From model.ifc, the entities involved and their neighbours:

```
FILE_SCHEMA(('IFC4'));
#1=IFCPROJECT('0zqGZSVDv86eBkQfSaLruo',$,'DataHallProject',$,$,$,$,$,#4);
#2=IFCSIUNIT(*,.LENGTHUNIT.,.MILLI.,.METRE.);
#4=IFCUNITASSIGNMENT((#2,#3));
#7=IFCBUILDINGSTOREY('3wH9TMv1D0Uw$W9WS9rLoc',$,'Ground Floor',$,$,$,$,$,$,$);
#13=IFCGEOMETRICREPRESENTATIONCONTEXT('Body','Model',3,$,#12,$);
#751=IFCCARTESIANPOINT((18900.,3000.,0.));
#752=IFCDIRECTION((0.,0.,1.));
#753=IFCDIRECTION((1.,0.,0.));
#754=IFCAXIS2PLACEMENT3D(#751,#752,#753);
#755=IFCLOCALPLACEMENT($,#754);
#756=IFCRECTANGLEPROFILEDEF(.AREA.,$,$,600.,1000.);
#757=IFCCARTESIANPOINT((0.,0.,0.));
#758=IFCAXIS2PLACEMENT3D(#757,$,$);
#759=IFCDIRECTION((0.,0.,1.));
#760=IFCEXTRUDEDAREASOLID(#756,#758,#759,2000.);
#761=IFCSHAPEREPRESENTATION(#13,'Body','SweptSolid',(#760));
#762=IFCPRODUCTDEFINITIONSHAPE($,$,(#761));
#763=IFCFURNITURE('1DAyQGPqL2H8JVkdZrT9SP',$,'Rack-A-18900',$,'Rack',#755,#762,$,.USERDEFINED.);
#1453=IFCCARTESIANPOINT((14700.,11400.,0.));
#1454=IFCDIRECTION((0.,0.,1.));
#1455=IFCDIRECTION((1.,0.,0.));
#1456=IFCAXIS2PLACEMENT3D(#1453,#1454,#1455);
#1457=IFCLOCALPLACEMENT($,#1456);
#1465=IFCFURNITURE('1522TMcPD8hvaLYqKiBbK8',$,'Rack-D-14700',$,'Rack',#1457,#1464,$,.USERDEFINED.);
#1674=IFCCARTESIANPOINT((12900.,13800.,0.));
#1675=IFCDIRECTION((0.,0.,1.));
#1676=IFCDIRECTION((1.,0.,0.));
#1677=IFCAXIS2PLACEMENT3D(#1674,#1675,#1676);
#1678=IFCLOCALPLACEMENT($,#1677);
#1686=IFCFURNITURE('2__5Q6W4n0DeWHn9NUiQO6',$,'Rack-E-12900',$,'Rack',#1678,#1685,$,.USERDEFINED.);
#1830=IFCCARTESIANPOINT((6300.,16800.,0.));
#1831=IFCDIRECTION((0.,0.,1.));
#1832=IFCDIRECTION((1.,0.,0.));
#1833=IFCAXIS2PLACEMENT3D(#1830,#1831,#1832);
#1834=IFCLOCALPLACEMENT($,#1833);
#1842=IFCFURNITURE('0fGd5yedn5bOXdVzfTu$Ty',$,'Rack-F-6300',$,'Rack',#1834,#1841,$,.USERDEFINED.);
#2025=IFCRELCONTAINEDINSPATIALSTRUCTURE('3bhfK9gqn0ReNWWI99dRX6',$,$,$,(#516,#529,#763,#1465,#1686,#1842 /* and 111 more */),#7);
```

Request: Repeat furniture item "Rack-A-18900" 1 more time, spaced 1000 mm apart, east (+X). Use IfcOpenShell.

```python
import numpy as np
import ifcopenshell
import ifcopenshell.api.geometry
import ifcopenshell.api.root
import ifcopenshell.util.element
import ifcopenshell.util.placement

model = ifcopenshell.open("model.ifc")

source = model.by_id(763)
base = ifcopenshell.util.placement.get_local_placement(source.ObjectPlacement)
step = np.array([1.0, 0.0, 0.0]) * 1000.0

for i in range(1, 2):
    copy = ifcopenshell.api.root.copy_class(model, product=source)
    copy.Representation = ifcopenshell.util.element.copy_deep(
        model, source.Representation, exclude=["IfcGeometricRepresentationContext", "IfcRepresentationMap"]
    )
    matrix = base.copy()
    matrix[:3, 3] += i * step
    print("added at", matrix[:3, 3].round(3) + 0.0)
    ifcopenshell.api.geometry.edit_object_placement(model, product=copy, matrix=matrix, is_si=False)

model.write("model_updated.ifc")
```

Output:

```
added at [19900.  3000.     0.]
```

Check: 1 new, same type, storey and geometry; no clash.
